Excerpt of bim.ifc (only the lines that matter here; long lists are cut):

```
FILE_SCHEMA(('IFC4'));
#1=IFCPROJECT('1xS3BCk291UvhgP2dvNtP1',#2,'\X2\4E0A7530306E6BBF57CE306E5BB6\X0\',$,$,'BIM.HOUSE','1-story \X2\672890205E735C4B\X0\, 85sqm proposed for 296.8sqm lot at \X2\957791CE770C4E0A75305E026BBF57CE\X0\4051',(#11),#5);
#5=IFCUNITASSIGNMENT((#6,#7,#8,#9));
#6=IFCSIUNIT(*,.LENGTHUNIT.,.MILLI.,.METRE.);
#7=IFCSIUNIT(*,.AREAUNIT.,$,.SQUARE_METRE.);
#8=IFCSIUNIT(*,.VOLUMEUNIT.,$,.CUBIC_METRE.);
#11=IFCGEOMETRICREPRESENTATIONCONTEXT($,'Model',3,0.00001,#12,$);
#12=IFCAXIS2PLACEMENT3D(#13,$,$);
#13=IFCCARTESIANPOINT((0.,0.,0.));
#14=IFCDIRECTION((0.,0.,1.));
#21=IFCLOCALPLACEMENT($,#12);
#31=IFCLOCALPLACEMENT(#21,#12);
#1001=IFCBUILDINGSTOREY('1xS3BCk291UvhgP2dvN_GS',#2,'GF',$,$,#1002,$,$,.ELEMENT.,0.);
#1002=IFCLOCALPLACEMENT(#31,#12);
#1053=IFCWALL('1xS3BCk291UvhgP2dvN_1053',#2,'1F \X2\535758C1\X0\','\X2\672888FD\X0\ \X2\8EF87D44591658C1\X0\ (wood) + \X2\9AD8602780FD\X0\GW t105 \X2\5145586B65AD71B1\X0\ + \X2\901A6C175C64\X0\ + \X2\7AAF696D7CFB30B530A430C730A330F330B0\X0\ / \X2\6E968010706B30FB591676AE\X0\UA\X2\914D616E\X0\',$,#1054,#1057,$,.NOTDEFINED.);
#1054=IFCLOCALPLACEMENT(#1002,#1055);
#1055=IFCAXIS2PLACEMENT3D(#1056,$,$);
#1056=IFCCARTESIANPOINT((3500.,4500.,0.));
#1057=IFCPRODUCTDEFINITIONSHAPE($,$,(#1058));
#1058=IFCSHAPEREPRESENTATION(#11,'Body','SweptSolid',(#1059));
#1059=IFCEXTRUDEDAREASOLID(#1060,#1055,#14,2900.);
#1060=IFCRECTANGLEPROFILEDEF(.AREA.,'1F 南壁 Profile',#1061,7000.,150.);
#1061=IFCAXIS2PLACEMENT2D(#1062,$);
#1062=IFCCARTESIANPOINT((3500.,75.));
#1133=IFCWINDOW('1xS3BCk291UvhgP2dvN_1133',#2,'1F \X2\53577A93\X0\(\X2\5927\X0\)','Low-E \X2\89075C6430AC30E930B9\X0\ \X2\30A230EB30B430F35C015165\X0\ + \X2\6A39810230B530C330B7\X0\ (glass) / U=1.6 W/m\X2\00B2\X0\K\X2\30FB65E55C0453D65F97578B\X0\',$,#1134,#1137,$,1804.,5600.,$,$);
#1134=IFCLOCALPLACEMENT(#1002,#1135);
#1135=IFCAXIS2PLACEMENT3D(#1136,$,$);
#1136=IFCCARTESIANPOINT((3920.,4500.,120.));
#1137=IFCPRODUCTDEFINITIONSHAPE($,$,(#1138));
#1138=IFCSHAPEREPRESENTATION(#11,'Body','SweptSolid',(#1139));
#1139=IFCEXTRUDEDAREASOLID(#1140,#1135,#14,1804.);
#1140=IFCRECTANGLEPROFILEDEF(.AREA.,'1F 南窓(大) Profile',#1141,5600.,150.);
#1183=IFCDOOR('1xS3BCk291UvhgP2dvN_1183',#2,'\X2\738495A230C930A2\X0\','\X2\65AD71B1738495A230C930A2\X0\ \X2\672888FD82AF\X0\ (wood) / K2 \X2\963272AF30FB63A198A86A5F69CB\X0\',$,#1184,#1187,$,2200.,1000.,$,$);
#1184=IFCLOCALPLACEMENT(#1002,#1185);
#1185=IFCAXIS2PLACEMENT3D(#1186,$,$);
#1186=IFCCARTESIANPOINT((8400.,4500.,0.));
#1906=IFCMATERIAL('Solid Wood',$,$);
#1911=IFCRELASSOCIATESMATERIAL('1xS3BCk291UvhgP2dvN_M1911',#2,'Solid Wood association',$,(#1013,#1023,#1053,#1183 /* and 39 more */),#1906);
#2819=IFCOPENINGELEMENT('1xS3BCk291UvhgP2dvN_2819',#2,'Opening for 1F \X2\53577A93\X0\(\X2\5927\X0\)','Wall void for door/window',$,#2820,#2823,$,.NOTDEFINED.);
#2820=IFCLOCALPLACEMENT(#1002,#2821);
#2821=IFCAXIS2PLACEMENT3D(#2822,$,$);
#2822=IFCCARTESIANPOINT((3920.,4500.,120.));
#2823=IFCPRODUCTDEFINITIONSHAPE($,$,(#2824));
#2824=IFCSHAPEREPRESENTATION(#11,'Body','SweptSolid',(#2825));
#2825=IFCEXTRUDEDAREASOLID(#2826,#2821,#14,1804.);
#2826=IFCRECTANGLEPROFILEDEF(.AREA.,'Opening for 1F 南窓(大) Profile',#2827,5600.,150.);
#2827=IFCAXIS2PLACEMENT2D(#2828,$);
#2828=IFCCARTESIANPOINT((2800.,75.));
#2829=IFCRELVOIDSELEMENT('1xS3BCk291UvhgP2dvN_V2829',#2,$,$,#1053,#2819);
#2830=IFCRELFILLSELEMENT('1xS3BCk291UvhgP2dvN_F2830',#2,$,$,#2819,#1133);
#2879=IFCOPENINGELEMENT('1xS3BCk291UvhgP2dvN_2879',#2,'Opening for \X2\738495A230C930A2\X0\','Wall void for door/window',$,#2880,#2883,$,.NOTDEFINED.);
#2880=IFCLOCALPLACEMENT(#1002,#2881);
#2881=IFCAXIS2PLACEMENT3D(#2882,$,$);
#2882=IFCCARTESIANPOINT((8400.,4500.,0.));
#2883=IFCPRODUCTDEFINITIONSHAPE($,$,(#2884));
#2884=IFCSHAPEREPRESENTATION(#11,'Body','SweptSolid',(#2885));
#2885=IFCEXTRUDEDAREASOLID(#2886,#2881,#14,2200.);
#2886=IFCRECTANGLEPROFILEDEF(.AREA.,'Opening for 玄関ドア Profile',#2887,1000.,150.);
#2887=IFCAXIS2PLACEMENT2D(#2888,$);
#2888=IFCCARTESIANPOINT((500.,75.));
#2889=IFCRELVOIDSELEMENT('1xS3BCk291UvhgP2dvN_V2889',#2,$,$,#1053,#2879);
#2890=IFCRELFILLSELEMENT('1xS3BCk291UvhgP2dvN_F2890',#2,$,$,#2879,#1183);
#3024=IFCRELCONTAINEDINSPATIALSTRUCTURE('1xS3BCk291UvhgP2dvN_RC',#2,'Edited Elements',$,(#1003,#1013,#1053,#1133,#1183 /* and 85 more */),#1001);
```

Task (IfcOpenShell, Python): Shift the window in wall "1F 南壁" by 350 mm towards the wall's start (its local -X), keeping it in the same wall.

```python
import ifcopenshell
import ifcopenshell.api.geometry
import ifcopenshell.util.placement
import ifcopenshell.util.unit

model = ifcopenshell.open("bim.ifc")
unit_scale = ifcopenshell.util.unit.calculate_unit_scale(model)

window = model.by_guid("1xS3BCk291UvhgP2dvN_1133")
opening = window.FillsVoids[0].RelatingOpeningElement
wall = opening.VoidsElements[0].RelatingBuildingElement

wall_matrix = ifcopenshell.util.placement.get_local_placement(wall.ObjectPlacement)
shift = wall_matrix[:3, 0] * -0.35 / unit_scale
before = ifcopenshell.util.placement.get_local_placement(window.ObjectPlacement)[:3, 3].copy()

# The window is not placed relative to its opening, so move both.
for product in (opening, window):
    matrix = ifcopenshell.util.placement.get_local_placement(product.ObjectPlacement)
    matrix[:3, 3] += shift
    ifcopenshell.api.geometry.edit_object_placement(model, product=product, matrix=matrix, is_si=False)

after = ifcopenshell.util.placement.get_local_placement(window.ObjectPlacement)[:3, 3]
print("window moved by", (after - before).round(3) + 0.0)

model.write("bim_updated.ifc")
```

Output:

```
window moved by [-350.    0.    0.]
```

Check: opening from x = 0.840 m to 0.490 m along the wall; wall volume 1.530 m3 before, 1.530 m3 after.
